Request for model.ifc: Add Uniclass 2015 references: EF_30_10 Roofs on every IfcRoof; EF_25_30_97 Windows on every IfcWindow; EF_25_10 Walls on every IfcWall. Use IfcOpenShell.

First a look at what the model holds.

```python
import ifcopenshell

model = ifcopenshell.open("model.ifc")
print(model.schema)
print("classifications:", [c.Name for c in model.by_type("IfcClassification")])
for ifc_class in ("IfcDoor", "IfcRoof", "IfcStair", "IfcWall", "IfcWindow"):
    print(ifc_class, len(model.by_type(ifc_class)))
```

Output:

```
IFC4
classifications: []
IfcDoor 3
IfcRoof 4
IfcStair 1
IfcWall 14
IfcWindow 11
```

```python
import ifcopenshell
import ifcopenshell.api.classification

model = ifcopenshell.open("model.ifc")

system = ifcopenshell.api.classification.add_classification(model, classification="Uniclass 2015")

codes = {
    "IfcRoof": ("EF_30_10", "Roofs"),
    "IfcWindow": ("EF_25_30_97", "Windows"),
    "IfcWall": ("EF_25_10", "Walls"),
}
for ifc_class, (code, name) in codes.items():
    products = model.by_type(ifc_class)
    ifcopenshell.api.classification.add_reference(
        model, products=products, classification=system, identification=code, name=name
    )
    print(code, len(products))

model.write("model-out.ifc")
```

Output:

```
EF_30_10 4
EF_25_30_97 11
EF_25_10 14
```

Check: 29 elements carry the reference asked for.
